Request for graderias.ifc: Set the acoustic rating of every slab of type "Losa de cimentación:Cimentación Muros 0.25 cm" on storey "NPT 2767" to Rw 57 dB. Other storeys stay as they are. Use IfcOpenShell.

First a look at what the model holds.

```python
import ifcopenshell
import ifcopenshell.util.element

model = ifcopenshell.open("graderias.ifc")
print(model.schema)
storey = next(s for s in model.by_type("IfcBuildingStorey") if s.Name == "NPT 2767")
slabs = [e for e in ifcopenshell.util.element.get_decomposition(storey) if e.is_a("IfcSlab")]
seen = {}
for e in slabs:
    element_type = ifcopenshell.util.element.get_type(e)
    key = (element_type.Name if element_type != e and element_type else None, ifcopenshell.util.element.get_pset(e, "Pset_SlabCommon", "AcousticRating"))
    seen[key] = seen.get(key, 0) + 1
for (name, value), count in sorted(seen.items(), key=str):
    print(count, "x", name, "|", value)
```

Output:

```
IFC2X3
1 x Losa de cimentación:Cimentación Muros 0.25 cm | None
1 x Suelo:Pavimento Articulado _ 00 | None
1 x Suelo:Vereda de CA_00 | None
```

```python
import ifcopenshell
import ifcopenshell.api.pset
import ifcopenshell.util.element

model = ifcopenshell.open("graderias.ifc")

storey = next(s for s in model.by_type("IfcBuildingStorey") if s.Name == "NPT 2767")
slabs = [e for e in ifcopenshell.util.element.get_decomposition(storey) if e.is_a("IfcSlab")]

count = 0
for e in slabs:
    element_type = ifcopenshell.util.element.get_type(e)
    if element_type in (None, e) or element_type.Name != "Losa de cimentación:Cimentación Muros 0.25 cm":
        continue
    # add_pset returns the element's existing set when there is one.
    pset = ifcopenshell.api.pset.add_pset(model, product=e, name="Pset_SlabCommon")
    ifcopenshell.api.pset.edit_pset(model, pset=pset, properties={"AcousticRating": "Rw 57 dB"})
    count += 1

print(count, "slabs updated")

model.write("graderias_v2.ifc")
```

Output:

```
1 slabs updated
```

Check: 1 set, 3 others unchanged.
